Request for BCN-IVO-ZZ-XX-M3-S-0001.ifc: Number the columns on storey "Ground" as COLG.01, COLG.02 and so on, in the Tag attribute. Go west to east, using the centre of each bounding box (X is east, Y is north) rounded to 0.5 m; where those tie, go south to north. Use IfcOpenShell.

First a look at what the model holds.

```python
import ifcopenshell
import ifcopenshell.util.element
import ifcopenshell.util.placement

model = ifcopenshell.open("BCN-IVO-ZZ-XX-M3-S-0001.ifc")
print(model.schema)
storey = next(s for s in model.by_type("IfcBuildingStorey") if s.Name == "Ground")
columns = [e for e in ifcopenshell.util.element.get_decomposition(storey) if e.is_a("IfcColumn")]
for e in sorted(columns, key=lambda e: e.id()):
    origin = ifcopenshell.util.placement.get_local_placement(e.ObjectPlacement)[:3, 3]
    print(e.id(), e.Tag, e.Name, origin.round(2) + 0.0, sep=" | ")
```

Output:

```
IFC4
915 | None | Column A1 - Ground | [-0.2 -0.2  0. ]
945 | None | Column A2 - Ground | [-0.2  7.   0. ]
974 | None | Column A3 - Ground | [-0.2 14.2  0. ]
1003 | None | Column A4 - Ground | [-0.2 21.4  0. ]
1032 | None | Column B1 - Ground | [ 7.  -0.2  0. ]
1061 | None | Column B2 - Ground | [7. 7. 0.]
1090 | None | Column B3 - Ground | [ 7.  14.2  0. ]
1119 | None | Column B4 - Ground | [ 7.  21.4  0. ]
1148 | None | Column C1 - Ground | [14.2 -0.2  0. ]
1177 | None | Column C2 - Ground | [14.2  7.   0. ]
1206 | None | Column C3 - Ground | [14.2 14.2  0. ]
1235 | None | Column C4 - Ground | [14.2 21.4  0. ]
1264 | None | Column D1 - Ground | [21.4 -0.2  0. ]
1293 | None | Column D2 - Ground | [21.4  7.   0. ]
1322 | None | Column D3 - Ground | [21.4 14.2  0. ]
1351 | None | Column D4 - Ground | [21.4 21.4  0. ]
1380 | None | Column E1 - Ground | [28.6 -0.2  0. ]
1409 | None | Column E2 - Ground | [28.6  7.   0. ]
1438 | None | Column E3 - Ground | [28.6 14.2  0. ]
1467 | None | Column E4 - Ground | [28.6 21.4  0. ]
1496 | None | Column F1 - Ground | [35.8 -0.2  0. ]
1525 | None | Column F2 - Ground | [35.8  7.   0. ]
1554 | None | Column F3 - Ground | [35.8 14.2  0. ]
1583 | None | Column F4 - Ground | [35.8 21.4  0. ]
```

```python
import ifcopenshell
import ifcopenshell.geom
import ifcopenshell.util.element
import ifcopenshell.util.shape

model = ifcopenshell.open("BCN-IVO-ZZ-XX-M3-S-0001.ifc")
settings = ifcopenshell.geom.settings()
settings.set("use-world-coords", True)


def centre(element):
    shape = ifcopenshell.geom.create_shape(settings, element)
    return ifcopenshell.util.shape.get_bbox_centroid(shape.geometry)


storey = next(s for s in model.by_type("IfcBuildingStorey") if s.Name == "Ground")
columns = [e for e in ifcopenshell.util.element.get_decomposition(storey) if e.is_a("IfcColumn")]

# Insertion points can sit at a corner or the storey origin, so sort by the geometry (in metres).
centres = {e: centre(e) for e in columns}
columns.sort(key=lambda e: (round(centres[e][0] / 0.5), centres[e][1]))

for i, e in enumerate(columns, start=1):
    number = f"COLG.{i:02d}"
    e.Tag = number
    print(e.id(), number)

model.write("BCN-IVO-ZZ-XX-M3-S-0001_v2.ifc")
```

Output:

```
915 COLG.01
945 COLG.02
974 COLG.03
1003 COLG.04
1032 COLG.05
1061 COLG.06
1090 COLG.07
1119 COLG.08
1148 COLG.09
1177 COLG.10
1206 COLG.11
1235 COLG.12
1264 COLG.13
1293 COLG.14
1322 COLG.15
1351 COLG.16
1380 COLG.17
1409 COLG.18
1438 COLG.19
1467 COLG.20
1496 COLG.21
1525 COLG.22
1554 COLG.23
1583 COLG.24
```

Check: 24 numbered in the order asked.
